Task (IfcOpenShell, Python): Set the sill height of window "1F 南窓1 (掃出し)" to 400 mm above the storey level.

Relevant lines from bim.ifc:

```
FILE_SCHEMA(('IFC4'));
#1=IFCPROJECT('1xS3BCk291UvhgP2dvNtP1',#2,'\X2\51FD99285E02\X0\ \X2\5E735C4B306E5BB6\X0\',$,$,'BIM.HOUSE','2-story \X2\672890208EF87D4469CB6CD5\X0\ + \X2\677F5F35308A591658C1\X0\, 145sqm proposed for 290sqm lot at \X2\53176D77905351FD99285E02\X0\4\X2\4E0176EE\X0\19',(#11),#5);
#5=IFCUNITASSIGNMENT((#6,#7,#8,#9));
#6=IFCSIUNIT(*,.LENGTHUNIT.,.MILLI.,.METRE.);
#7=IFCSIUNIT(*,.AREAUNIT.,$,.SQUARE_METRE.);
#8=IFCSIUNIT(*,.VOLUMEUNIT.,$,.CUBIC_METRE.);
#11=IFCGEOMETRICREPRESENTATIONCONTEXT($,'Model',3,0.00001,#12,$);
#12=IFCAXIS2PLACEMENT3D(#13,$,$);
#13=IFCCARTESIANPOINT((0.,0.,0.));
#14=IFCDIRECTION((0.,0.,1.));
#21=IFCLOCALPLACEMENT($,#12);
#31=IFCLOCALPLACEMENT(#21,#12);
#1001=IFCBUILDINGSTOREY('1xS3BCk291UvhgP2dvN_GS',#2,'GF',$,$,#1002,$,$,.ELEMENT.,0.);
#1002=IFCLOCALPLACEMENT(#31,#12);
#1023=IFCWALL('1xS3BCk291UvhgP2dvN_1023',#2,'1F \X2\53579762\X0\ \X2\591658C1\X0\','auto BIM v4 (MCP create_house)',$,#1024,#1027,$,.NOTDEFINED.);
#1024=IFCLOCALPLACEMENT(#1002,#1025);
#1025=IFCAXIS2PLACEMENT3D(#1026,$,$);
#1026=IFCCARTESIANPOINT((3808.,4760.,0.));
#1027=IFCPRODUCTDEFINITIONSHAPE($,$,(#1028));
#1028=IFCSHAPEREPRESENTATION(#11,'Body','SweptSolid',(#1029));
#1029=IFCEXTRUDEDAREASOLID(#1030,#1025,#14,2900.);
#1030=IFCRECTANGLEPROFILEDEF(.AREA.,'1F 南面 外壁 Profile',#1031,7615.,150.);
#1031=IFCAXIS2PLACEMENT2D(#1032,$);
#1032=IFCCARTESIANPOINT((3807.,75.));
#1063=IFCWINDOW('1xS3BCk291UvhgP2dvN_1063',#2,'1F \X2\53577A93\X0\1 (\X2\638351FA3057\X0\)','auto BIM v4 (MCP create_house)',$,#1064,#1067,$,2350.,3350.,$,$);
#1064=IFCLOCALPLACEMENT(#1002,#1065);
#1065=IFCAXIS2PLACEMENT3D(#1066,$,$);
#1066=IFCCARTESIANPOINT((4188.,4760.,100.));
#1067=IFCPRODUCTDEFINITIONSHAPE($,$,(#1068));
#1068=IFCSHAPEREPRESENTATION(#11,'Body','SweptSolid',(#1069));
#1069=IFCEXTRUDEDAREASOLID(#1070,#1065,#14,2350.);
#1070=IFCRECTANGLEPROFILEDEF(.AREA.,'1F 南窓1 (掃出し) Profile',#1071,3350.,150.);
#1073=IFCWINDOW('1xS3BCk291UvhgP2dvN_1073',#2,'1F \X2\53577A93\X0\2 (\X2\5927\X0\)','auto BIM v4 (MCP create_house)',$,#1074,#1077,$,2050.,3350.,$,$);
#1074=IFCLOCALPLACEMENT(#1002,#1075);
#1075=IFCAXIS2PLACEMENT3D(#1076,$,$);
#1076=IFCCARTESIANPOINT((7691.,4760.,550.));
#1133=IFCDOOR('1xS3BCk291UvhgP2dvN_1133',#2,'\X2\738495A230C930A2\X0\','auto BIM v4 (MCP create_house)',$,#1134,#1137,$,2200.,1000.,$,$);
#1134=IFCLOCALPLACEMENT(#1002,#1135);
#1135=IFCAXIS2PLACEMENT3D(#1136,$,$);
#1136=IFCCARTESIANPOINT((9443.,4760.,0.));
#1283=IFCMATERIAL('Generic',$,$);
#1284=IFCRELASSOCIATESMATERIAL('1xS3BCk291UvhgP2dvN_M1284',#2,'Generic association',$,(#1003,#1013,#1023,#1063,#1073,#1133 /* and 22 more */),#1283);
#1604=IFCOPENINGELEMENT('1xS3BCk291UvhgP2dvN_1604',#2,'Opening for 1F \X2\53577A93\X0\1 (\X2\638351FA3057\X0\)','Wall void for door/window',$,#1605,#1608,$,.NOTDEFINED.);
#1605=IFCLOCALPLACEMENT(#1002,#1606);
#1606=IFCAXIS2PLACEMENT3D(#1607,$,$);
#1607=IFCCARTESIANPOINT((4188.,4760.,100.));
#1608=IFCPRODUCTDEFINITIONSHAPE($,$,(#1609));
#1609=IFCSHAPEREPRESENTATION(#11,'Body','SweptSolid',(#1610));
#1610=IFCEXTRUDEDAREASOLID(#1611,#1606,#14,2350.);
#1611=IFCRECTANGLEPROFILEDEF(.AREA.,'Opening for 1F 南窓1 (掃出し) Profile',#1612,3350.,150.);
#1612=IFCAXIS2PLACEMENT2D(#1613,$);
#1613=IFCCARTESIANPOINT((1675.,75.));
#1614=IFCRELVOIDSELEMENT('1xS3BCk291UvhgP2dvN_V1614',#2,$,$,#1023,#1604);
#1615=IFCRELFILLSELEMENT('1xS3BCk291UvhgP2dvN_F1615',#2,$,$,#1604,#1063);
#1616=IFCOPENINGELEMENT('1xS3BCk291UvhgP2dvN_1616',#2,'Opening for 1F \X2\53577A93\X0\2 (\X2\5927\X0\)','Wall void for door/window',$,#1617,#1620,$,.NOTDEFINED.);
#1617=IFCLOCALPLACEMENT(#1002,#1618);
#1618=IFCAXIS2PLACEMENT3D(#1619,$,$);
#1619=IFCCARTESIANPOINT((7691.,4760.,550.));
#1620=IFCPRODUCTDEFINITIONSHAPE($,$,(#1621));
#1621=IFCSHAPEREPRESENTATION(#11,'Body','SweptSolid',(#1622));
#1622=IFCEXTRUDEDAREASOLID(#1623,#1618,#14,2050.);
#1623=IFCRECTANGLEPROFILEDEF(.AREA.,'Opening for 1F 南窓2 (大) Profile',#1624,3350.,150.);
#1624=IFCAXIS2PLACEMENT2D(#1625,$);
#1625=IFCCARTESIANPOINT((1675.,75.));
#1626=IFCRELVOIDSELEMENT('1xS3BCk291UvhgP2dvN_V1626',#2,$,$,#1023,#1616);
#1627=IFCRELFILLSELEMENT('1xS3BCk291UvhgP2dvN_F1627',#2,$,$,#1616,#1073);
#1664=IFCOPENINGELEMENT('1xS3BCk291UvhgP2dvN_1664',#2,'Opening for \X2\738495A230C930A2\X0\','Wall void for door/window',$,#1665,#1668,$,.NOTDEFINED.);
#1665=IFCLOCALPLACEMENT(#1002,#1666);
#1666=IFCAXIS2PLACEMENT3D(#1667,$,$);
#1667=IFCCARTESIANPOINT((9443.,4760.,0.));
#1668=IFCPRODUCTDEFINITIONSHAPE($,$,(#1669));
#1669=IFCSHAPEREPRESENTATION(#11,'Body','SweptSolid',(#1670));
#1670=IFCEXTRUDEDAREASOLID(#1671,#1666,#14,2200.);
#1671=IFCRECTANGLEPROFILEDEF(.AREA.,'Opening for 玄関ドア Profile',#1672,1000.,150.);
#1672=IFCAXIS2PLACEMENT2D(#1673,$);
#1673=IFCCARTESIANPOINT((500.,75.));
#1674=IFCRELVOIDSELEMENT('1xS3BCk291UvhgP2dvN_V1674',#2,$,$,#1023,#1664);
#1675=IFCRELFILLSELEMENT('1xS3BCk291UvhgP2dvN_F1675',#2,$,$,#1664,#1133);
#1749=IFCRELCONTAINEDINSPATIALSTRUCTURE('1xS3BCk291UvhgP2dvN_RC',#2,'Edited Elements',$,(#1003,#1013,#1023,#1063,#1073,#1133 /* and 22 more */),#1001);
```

```python
import numpy as np
import ifcopenshell
import ifcopenshell.api.geometry
import ifcopenshell.geom
import ifcopenshell.util.element
import ifcopenshell.util.placement
import ifcopenshell.util.shape
import ifcopenshell.util.unit

model = ifcopenshell.open("bim.ifc")
unit_scale = ifcopenshell.util.unit.calculate_unit_scale(model)

window = model.by_guid("1xS3BCk291UvhgP2dvN_1063")
opening = window.FillsVoids[0].RelatingOpeningElement
storey = ifcopenshell.util.element.get_container(window, ifc_class="IfcBuildingStorey")
level = ifcopenshell.util.placement.get_local_placement(storey.ObjectPlacement)[2, 3]

# The opening's origin need not be at the sill, so measure its lowest point.
shape = ifcopenshell.geom.create_shape(ifcopenshell.geom.settings(), opening)
bottom = ifcopenshell.util.shape.get_shape_bottom_elevation(shape, shape.geometry) / unit_scale
dz = level + 400.0 - bottom

shift = np.array([0.0, 0.0, dz])
# The window is not placed relative to its opening, so move both.
for product in (opening, window):
    matrix = ifcopenshell.util.placement.get_local_placement(product.ObjectPlacement)
    matrix[:3, 3] += shift
    ifcopenshell.api.geometry.edit_object_placement(model, product=product, matrix=matrix, is_si=False)

print(f"moved by {dz * unit_scale:+.3f} m")

model.write("bim_rev.ifc")
```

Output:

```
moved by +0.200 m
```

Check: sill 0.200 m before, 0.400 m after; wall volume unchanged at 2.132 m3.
